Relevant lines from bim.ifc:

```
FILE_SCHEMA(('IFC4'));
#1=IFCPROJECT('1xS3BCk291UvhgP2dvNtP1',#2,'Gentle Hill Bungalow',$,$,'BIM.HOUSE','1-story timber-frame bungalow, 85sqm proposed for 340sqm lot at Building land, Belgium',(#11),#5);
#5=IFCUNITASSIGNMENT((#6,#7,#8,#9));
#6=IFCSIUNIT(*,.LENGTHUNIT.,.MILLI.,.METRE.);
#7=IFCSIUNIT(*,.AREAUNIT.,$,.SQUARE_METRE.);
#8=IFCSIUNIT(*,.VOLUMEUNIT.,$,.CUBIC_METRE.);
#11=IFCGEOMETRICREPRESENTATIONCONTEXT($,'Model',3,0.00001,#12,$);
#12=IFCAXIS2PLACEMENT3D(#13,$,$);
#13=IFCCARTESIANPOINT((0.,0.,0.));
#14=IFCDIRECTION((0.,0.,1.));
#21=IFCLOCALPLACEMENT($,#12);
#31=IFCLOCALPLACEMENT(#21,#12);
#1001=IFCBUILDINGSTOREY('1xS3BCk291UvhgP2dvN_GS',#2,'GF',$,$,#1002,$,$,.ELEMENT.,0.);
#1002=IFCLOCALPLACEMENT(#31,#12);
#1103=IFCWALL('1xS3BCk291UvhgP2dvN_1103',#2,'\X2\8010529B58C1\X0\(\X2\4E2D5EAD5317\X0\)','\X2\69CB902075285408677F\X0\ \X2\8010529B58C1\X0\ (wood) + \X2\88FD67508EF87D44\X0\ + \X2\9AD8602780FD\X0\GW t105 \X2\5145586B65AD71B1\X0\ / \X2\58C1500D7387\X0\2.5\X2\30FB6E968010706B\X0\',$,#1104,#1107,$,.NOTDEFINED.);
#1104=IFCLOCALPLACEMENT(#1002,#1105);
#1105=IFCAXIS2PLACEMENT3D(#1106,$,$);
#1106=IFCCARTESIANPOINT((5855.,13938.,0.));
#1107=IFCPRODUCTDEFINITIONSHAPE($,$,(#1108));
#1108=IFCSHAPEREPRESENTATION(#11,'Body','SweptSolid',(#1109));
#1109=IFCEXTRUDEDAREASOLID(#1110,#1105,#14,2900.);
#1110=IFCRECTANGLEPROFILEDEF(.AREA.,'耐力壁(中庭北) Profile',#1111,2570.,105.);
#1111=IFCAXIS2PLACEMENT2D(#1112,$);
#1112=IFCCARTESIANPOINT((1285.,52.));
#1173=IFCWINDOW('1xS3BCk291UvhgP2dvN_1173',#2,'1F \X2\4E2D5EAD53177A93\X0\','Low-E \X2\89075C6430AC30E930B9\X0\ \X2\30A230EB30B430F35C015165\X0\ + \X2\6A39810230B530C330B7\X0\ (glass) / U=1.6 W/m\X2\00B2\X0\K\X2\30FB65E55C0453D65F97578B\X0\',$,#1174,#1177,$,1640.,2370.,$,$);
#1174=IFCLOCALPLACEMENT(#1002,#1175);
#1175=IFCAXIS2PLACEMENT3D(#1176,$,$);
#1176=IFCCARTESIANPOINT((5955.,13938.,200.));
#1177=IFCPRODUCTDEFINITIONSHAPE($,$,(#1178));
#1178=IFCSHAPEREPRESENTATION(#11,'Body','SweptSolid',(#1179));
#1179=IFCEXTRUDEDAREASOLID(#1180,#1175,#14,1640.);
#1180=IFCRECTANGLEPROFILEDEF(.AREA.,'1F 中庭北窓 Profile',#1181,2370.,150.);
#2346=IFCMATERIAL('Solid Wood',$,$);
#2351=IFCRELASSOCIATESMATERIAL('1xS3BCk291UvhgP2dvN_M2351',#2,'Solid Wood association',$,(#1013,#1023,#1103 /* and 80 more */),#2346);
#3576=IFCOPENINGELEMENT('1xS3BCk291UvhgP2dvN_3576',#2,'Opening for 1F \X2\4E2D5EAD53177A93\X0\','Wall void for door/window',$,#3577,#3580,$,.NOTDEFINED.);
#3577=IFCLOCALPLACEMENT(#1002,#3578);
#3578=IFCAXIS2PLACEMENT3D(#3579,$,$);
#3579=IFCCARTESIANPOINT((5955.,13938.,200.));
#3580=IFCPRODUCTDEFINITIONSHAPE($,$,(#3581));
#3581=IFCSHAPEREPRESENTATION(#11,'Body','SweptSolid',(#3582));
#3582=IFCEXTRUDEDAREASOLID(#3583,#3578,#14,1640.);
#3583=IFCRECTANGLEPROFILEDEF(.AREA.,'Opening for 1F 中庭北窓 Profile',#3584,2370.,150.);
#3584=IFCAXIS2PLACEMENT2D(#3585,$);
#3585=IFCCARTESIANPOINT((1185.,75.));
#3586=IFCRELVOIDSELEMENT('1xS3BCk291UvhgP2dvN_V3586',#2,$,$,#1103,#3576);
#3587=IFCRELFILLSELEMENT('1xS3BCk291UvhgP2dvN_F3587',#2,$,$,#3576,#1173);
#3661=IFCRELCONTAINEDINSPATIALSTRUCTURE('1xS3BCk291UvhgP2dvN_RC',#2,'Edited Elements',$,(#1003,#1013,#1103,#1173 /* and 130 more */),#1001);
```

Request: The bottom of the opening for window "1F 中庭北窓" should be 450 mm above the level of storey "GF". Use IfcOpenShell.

```python
import numpy as np
import ifcopenshell
import ifcopenshell.api.geometry
import ifcopenshell.geom
import ifcopenshell.util.element
import ifcopenshell.util.placement
import ifcopenshell.util.shape
import ifcopenshell.util.unit

model = ifcopenshell.open("bim.ifc")
unit_scale = ifcopenshell.util.unit.calculate_unit_scale(model)

window = model.by_guid("1xS3BCk291UvhgP2dvN_1173")
opening = window.FillsVoids[0].RelatingOpeningElement
storey = ifcopenshell.util.element.get_container(window, ifc_class="IfcBuildingStorey")
level = ifcopenshell.util.placement.get_local_placement(storey.ObjectPlacement)[2, 3]

# The opening's origin need not be at the sill, so measure its lowest point.
shape = ifcopenshell.geom.create_shape(ifcopenshell.geom.settings(), opening)
bottom = ifcopenshell.util.shape.get_shape_bottom_elevation(shape, shape.geometry) / unit_scale
dz = level + 0.45 / unit_scale - bottom

shift = np.array([0.0, 0.0, dz])
# The window is not placed relative to its opening, so move both.
for product in (opening, window):
    matrix = ifcopenshell.util.placement.get_local_placement(product.ObjectPlacement)
    matrix[:3, 3] += shift
    ifcopenshell.api.geometry.edit_object_placement(model, product=product, matrix=matrix, is_si=False)

print(f"moved by {dz * unit_scale:+.3f} m")

model.write("bim-out.ifc")
```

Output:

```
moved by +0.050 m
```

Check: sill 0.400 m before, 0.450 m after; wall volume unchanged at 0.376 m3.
